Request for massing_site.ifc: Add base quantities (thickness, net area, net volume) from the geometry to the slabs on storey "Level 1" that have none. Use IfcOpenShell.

First a look at what the model holds.

```python
import ifcopenshell
import ifcopenshell.util.element
import ifcopenshell.util.unit

model = ifcopenshell.open("massing_site.ifc")
print(model.schema)
for unit_type in ("LENGTHUNIT", "AREAUNIT", "VOLUMEUNIT"):
    print(unit_type, ifcopenshell.util.unit.calculate_unit_scale(model, unit_type))
storey = next(s for s in model.by_type("IfcBuildingStorey") if s.Name == "Level 1")
slabs = [e for e in ifcopenshell.util.element.get_decomposition(storey) if e.is_a("IfcSlab")]
for e in sorted(slabs, key=lambda e: e.id()):
    print(e.id(), e.is_a(), e.Name, list(ifcopenshell.util.element.get_psets(e, qtos_only=True)), sep=" | ")
```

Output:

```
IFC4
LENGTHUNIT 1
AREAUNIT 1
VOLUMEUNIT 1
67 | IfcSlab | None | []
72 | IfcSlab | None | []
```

```python
import ifcopenshell
import ifcopenshell.api.pset
import ifcopenshell.geom
import ifcopenshell.util.element
import ifcopenshell.util.shape
import ifcopenshell.util.unit

model = ifcopenshell.open("massing_site.ifc")
unit_scale = ifcopenshell.util.unit.calculate_unit_scale(model)
area_scale = ifcopenshell.util.unit.calculate_unit_scale(model, "AREAUNIT")
volume_scale = ifcopenshell.util.unit.calculate_unit_scale(model, "VOLUMEUNIT")
settings = ifcopenshell.geom.settings()

storey = next(s for s in model.by_type("IfcBuildingStorey") if s.Name == "Level 1")
slabs = [e for e in ifcopenshell.util.element.get_decomposition(storey) if e.is_a("IfcSlab")]

for e in sorted(slabs, key=lambda e: e.id()):
    if ifcopenshell.util.element.get_psets(e, qtos_only=True, should_inherit=False):
        continue
    # Geometry comes back in metres, in the element's own axes.
    shape = ifcopenshell.geom.create_shape(settings, e)
    values = {
        "Width": ifcopenshell.util.shape.get_z(shape.geometry) / unit_scale,
        "NetArea": ifcopenshell.util.shape.get_footprint_area(shape.geometry) / area_scale,
        "NetVolume": ifcopenshell.util.shape.get_volume(shape.geometry) / volume_scale,
    }
    qto = ifcopenshell.api.pset.add_qto(model, product=e, name="Qto_SlabBaseQuantities")
    ifcopenshell.api.pset.edit_qto(model, qto=qto, properties=values)
    print(e.id(), {k: round(v, 3) for k, v in values.items()})

model.write("massing_site_v2.ifc")
```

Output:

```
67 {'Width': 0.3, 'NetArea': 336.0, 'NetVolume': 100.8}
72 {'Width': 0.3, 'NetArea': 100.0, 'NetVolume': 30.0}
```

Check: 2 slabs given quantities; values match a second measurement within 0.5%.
